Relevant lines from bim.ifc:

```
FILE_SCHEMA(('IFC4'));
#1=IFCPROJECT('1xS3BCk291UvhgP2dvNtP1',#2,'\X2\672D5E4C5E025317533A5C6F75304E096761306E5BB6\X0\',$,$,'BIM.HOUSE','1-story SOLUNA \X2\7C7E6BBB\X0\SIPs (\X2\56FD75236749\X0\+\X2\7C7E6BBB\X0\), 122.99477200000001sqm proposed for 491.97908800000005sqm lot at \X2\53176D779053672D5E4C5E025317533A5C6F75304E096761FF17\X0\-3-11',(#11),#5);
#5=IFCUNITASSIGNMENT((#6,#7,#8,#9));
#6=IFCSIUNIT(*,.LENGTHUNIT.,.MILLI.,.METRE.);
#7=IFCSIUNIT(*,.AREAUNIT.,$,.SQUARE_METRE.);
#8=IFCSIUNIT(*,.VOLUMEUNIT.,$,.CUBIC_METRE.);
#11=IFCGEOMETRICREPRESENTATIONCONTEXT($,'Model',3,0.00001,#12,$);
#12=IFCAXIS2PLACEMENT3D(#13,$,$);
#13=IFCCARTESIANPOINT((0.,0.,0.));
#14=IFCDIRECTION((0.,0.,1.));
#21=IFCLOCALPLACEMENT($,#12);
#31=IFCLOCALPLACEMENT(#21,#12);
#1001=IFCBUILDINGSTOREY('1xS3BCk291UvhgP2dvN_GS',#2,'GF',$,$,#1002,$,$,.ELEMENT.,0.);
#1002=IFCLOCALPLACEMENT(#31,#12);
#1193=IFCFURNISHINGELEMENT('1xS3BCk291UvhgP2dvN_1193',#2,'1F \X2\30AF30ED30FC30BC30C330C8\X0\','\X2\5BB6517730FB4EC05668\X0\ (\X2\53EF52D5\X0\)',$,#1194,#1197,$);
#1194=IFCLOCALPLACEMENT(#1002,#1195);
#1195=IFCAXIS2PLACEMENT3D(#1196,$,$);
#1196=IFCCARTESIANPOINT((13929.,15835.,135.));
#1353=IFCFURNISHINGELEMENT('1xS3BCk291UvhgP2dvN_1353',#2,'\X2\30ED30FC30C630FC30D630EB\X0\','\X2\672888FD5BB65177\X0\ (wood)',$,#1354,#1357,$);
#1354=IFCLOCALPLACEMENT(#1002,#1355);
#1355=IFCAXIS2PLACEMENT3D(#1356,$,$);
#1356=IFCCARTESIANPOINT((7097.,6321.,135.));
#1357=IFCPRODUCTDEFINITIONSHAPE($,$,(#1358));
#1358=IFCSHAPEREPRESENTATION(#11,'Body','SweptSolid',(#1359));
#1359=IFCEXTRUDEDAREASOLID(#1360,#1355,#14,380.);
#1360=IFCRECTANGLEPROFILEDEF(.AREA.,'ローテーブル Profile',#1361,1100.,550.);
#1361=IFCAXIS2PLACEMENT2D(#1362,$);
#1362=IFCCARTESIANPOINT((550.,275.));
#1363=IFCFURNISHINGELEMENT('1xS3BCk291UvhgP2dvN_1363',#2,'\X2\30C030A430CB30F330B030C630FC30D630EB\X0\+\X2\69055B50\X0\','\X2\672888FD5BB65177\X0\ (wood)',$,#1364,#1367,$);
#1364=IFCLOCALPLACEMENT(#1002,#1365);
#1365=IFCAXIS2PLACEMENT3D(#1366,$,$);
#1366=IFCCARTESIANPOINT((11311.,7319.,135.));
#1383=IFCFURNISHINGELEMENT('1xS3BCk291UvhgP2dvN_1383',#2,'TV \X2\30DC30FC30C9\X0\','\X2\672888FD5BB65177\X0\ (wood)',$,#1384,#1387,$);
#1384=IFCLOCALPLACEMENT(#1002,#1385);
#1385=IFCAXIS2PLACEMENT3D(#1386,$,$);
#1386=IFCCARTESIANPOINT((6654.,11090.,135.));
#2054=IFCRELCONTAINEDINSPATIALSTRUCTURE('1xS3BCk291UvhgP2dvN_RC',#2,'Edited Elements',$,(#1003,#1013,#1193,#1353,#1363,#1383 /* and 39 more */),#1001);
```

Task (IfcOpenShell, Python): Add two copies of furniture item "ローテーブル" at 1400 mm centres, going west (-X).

```python
import numpy as np
import ifcopenshell
import ifcopenshell.api.geometry
import ifcopenshell.api.root
import ifcopenshell.util.element
import ifcopenshell.util.placement

model = ifcopenshell.open("bim.ifc")


def reuse_history(source, copy):
    """copy_class also copies each property set's owner history, people and application; keep the originals."""
    for rel in copy.IsDefinedBy:
        if rel.is_a("IfcRelDefinesByProperties") and (history := rel.RelatingPropertyDefinition.OwnerHistory):
            rel.RelatingPropertyDefinition.OwnerHistory = source.OwnerHistory
            ifcopenshell.util.element.remove_deep2(model, history)


source = model.by_guid("1xS3BCk291UvhgP2dvN_1353")
base = ifcopenshell.util.placement.get_local_placement(source.ObjectPlacement)
step = np.array([-1.0, 0.0, 0.0]) * 1400.0

for i in range(1, 3):
    copy = ifcopenshell.api.root.copy_class(model, product=source)
    copy.Representation = ifcopenshell.util.element.copy_deep(
        model, source.Representation, exclude=["IfcGeometricRepresentationContext", "IfcRepresentationMap"]
    )
    reuse_history(source, copy)
    matrix = base.copy()
    matrix[:3, 3] += i * step
    print("added at", matrix[:3, 3].round(3) + 0.0)
    ifcopenshell.api.geometry.edit_object_placement(model, product=copy, matrix=matrix, is_si=False)

model.write("bim_v2.ifc")
```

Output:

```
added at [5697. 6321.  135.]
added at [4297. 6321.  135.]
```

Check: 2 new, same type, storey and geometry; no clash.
